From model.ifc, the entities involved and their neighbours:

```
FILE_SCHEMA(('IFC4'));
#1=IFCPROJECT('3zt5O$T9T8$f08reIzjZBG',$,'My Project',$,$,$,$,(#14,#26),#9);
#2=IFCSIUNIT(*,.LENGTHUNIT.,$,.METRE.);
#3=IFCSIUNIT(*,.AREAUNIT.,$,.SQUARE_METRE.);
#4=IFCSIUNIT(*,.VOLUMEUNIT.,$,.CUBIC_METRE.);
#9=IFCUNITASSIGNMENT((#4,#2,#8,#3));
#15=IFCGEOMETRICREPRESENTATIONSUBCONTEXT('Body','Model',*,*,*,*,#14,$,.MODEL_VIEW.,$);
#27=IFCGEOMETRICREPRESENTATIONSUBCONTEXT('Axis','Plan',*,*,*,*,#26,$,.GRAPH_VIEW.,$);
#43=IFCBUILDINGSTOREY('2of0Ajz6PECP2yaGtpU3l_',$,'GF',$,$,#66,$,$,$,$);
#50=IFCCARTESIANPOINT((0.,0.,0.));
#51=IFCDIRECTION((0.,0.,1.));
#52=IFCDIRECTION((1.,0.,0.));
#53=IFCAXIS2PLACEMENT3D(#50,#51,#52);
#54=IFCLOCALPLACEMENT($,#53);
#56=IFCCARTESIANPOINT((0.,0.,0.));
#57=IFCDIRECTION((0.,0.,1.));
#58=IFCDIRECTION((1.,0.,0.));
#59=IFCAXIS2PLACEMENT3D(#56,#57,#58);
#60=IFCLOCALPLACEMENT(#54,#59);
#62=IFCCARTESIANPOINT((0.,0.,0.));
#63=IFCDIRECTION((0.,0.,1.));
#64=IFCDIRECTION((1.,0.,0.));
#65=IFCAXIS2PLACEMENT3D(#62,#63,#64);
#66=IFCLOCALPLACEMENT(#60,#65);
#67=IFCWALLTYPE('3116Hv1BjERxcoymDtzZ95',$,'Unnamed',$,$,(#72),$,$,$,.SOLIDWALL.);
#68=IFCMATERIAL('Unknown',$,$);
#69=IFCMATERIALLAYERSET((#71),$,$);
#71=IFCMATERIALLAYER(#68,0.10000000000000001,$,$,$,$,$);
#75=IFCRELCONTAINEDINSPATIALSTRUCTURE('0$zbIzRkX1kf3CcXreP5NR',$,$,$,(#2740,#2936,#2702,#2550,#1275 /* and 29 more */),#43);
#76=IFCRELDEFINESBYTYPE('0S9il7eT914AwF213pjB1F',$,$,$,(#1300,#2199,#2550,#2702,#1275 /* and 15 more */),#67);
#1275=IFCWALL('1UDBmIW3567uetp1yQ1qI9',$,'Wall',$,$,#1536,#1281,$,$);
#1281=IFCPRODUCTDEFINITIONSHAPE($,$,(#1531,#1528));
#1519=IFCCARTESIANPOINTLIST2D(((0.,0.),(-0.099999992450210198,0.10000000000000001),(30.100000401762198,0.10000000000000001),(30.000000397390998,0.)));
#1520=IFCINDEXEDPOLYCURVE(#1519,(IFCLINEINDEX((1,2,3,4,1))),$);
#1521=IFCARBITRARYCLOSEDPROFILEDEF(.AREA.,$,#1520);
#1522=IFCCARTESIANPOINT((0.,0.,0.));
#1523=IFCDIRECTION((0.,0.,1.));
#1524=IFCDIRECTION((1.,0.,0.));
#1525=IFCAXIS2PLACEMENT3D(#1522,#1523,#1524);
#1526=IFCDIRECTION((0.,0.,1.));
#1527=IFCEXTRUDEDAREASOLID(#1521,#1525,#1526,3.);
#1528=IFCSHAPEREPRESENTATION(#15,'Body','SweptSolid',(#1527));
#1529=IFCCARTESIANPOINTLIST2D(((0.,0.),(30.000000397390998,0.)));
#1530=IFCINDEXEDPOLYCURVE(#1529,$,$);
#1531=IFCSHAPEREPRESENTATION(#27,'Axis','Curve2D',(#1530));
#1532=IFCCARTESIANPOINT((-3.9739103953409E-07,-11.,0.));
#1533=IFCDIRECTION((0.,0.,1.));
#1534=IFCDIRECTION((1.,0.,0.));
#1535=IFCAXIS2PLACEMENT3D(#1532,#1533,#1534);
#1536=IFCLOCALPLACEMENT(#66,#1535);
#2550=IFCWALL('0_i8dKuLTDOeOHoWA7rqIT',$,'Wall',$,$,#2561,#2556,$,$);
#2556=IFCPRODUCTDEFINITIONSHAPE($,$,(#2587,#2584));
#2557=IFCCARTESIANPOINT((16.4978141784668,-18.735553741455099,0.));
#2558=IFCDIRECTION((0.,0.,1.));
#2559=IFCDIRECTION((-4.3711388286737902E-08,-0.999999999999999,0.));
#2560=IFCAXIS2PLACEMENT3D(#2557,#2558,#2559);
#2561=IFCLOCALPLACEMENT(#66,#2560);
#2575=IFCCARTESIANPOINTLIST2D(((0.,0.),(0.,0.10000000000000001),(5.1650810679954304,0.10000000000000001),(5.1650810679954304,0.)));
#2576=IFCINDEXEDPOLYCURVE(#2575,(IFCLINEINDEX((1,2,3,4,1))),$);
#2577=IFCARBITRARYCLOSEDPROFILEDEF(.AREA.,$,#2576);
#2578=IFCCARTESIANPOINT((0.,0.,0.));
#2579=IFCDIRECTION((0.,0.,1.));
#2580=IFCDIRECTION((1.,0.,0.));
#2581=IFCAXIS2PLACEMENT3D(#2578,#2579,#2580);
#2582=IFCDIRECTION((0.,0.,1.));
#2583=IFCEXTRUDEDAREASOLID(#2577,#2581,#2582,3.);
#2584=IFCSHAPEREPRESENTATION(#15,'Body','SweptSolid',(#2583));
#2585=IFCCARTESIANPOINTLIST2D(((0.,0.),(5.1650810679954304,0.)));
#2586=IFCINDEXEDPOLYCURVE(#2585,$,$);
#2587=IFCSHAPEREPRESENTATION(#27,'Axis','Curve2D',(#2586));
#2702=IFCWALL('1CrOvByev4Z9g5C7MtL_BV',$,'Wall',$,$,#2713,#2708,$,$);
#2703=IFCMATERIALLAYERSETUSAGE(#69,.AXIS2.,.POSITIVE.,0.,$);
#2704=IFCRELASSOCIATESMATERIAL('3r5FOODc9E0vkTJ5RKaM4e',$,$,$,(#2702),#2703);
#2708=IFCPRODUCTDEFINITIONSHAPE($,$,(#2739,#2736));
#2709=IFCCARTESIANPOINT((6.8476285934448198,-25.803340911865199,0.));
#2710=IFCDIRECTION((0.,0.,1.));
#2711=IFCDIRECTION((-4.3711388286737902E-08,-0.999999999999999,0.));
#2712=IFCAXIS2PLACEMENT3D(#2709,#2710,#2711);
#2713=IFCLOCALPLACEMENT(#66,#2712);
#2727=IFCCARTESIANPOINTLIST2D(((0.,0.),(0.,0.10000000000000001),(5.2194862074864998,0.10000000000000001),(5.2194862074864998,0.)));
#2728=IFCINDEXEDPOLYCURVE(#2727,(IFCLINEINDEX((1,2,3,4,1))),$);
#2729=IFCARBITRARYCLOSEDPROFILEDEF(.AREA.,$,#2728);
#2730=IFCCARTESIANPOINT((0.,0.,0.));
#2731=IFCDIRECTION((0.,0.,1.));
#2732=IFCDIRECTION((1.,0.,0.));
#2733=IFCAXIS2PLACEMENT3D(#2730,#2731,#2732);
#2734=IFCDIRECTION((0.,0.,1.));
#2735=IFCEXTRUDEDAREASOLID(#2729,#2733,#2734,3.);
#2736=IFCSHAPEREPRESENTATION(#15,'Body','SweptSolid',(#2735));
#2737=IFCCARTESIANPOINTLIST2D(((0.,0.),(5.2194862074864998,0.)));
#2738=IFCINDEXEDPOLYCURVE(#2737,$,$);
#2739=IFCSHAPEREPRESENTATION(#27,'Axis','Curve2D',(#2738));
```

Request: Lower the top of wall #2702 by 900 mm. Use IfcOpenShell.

```python
import ifcopenshell
import ifcopenshell.geom
import ifcopenshell.util.representation
import ifcopenshell.util.shape
import ifcopenshell.util.unit

model = ifcopenshell.open("model.ifc")
unit_scale = ifcopenshell.util.unit.calculate_unit_scale(model)
settings = ifcopenshell.geom.settings()


def volume(element):
    """Net volume in cubic metres, openings subtracted."""
    shape = ifcopenshell.geom.create_shape(settings, element)
    return ifcopenshell.util.shape.get_volume(shape.geometry)


wall = model.by_guid("1CrOvByev4Z9g5C7MtL_BV")
before = volume(wall)

body = ifcopenshell.util.representation.get_representation(wall, "Model", "Body")
solid = body.Items[0]
old_height = solid.Depth
solid.Depth -= 0.9 / unit_scale
after = volume(wall)

print(f"height {old_height:g} -> {solid.Depth:g}, volume {before:.3f} -> {after:.3f} m3")

model.write("model-out.ifc")
```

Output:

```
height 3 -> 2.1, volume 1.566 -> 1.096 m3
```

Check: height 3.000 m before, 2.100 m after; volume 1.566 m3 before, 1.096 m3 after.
